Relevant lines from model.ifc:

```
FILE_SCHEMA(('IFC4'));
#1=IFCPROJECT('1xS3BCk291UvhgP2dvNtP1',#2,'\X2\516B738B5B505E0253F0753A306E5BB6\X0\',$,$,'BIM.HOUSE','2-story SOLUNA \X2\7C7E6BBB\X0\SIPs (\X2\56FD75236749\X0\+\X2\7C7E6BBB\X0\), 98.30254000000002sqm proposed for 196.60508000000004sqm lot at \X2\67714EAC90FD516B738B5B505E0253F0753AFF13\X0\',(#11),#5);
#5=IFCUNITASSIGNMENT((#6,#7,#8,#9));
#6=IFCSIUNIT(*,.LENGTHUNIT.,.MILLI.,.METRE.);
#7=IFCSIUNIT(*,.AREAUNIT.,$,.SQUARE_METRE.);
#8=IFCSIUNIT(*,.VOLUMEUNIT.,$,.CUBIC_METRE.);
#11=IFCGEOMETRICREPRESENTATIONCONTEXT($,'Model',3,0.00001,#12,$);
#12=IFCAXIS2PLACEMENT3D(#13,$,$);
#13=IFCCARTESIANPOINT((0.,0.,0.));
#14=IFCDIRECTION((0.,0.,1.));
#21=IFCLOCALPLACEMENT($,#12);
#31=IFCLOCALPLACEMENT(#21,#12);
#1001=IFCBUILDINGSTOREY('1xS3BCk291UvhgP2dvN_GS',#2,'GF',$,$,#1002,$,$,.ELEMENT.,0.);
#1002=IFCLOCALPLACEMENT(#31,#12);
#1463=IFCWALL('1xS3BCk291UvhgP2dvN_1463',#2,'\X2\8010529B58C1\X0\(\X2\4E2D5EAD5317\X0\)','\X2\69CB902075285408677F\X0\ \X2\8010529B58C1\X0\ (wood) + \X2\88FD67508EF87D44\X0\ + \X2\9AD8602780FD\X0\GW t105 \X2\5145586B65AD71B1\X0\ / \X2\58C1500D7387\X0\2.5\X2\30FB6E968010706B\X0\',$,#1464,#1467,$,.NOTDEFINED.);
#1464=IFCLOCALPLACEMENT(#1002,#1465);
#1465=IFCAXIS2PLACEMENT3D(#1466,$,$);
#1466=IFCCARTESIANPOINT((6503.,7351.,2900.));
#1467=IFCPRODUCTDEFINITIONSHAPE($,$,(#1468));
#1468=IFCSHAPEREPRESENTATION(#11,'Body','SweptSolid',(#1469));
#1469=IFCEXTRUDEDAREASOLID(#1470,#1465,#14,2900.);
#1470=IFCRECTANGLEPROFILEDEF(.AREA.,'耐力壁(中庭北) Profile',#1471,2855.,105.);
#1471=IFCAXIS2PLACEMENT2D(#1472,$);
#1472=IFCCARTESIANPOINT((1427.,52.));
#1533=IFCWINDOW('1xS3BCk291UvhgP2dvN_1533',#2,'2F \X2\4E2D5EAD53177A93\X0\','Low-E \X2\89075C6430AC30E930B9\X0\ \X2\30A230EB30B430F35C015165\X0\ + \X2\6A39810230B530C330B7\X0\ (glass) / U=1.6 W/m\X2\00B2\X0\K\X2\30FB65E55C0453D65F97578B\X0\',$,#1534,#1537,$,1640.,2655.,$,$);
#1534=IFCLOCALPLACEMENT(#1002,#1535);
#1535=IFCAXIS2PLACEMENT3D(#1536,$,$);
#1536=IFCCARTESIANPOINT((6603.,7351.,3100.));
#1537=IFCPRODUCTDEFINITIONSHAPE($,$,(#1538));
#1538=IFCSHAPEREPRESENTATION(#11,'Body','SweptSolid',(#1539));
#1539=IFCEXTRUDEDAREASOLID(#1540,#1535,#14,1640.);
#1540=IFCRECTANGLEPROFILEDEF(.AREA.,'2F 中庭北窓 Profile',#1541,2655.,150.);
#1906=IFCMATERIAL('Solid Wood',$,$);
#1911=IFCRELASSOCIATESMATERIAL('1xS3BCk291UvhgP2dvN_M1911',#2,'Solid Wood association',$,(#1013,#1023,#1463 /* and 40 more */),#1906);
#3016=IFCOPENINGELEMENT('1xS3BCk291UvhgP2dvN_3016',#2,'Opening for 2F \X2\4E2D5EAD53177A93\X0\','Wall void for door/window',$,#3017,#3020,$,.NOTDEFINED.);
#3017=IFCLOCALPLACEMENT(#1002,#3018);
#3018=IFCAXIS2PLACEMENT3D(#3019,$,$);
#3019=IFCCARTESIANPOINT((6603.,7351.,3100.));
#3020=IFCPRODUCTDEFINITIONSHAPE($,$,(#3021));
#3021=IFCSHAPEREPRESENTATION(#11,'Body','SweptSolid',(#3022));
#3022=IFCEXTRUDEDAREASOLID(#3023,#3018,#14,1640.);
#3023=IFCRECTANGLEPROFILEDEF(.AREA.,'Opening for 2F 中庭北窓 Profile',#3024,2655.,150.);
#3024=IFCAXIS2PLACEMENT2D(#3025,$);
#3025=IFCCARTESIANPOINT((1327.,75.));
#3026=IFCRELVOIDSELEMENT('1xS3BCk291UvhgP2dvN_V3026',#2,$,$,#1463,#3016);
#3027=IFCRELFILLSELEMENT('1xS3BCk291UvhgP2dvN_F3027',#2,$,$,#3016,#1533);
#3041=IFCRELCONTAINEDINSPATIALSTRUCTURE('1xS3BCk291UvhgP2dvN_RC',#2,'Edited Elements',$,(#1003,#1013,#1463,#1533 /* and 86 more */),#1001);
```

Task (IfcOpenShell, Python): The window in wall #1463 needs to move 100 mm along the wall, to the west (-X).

```python
import ifcopenshell
import ifcopenshell.api.geometry
import ifcopenshell.util.placement
import ifcopenshell.util.unit

model = ifcopenshell.open("model.ifc")
unit_scale = ifcopenshell.util.unit.calculate_unit_scale(model)

window = model.by_id(1533)
opening = window.FillsVoids[0].RelatingOpeningElement
wall = opening.VoidsElements[0].RelatingBuildingElement

wall_matrix = ifcopenshell.util.placement.get_local_placement(wall.ObjectPlacement)
shift = wall_matrix[:3, 0] * -0.1 / unit_scale
before = ifcopenshell.util.placement.get_local_placement(window.ObjectPlacement)[:3, 3].copy()

# The window is not placed relative to its opening, so move both.
for product in (opening, window):
    matrix = ifcopenshell.util.placement.get_local_placement(product.ObjectPlacement)
    matrix[:3, 3] += shift
    ifcopenshell.api.geometry.edit_object_placement(model, product=product, matrix=matrix, is_si=False)

after = ifcopenshell.util.placement.get_local_placement(window.ObjectPlacement)[:3, 3]
print("window moved by", (after - before).round(3) + 0.0)

model.write("model_edited.ifc")
```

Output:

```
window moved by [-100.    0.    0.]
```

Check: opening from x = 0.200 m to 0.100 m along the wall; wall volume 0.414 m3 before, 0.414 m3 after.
